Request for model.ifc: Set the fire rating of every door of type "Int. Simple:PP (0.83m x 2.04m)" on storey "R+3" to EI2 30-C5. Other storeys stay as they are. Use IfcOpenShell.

First a look at what the model holds.

```python
import ifcopenshell
import ifcopenshell.util.element

model = ifcopenshell.open("model.ifc")
print(model.schema)
storey = next(s for s in model.by_type("IfcBuildingStorey") if s.Name == "R+3")
doors = [e for e in ifcopenshell.util.element.get_decomposition(storey) if e.is_a("IfcDoor")]
seen = {}
for e in doors:
    element_type = ifcopenshell.util.element.get_type(e)
    key = (element_type.Name if element_type != e and element_type else None, ifcopenshell.util.element.get_pset(e, "Pset_DoorCommon", "FireRating"))
    seen[key] = seen.get(key, 0) + 1
for (name, value), count in sorted(seen.items(), key=str):
    print(count, "x", name, "|", value)
```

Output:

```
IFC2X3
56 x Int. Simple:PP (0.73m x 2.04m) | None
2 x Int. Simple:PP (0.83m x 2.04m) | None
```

```python
import ifcopenshell
import ifcopenshell.api.pset
import ifcopenshell.util.element

model = ifcopenshell.open("model.ifc")

storey = next(s for s in model.by_type("IfcBuildingStorey") if s.Name == "R+3")
doors = [e for e in ifcopenshell.util.element.get_decomposition(storey) if e.is_a("IfcDoor")]

count = 0
for e in doors:
    element_type = ifcopenshell.util.element.get_type(e)
    if element_type in (None, e) or element_type.Name != "Int. Simple:PP (0.83m x 2.04m)":
        continue
    # add_pset returns the element's existing set when there is one.
    pset = ifcopenshell.api.pset.add_pset(model, product=e, name="Pset_DoorCommon")
    ifcopenshell.api.pset.edit_pset(model, pset=pset, properties={"FireRating": "EI2 30-C5"})
    count += 1

print(count, "doors updated")

model.write("model_v2.ifc")
```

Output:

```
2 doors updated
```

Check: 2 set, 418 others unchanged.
